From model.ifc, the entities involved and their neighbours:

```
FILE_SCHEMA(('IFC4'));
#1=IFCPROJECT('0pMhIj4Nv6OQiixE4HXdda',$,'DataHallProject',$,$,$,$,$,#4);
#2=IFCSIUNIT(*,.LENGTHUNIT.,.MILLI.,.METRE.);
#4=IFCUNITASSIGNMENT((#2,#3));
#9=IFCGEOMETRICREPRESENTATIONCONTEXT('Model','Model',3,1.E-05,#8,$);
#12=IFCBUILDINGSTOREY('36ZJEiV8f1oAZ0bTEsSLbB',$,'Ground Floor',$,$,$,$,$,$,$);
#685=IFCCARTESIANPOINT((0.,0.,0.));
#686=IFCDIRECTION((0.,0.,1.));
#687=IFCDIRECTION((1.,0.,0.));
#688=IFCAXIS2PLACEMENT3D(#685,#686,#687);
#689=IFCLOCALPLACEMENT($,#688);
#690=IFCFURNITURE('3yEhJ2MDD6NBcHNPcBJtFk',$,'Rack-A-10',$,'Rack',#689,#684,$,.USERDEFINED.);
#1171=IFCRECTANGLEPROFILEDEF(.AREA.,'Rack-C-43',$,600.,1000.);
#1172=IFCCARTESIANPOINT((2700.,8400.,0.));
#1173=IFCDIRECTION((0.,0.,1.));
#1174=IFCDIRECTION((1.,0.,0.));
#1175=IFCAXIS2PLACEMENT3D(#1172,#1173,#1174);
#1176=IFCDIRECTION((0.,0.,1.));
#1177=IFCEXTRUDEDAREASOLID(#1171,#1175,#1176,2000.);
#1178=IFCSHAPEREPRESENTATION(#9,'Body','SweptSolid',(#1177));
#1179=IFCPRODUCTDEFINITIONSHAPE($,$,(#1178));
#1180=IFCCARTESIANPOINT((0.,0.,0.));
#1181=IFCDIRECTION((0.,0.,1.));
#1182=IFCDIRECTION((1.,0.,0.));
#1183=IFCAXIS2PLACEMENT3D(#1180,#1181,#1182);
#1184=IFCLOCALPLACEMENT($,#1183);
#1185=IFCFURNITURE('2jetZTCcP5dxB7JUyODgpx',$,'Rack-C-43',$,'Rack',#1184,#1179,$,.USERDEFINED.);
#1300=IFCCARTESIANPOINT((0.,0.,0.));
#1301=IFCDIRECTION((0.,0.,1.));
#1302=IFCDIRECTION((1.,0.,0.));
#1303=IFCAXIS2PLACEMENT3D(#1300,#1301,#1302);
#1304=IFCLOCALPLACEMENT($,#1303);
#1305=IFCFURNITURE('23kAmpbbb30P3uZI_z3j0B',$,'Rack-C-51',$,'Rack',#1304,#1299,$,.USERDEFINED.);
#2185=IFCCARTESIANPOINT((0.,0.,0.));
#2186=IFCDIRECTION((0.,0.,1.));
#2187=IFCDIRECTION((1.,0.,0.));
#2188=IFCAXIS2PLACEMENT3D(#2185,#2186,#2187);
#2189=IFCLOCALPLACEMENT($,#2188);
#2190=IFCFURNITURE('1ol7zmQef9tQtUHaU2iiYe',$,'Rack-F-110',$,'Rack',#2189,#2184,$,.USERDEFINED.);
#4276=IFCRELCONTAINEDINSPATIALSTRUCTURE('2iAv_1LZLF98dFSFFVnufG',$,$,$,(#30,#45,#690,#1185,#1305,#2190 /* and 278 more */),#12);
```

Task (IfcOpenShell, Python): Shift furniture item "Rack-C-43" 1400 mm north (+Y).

```python
import ifcopenshell
import ifcopenshell.api.geometry
import ifcopenshell.util.placement
import ifcopenshell.util.unit

model = ifcopenshell.open("model.ifc")
unit_scale = ifcopenshell.util.unit.calculate_unit_scale(model)

item = model.by_guid("2jetZTCcP5dxB7JUyODgpx")
matrix = ifcopenshell.util.placement.get_local_placement(item.ObjectPlacement)
matrix[1, 3] += 1.4 / unit_scale
ifcopenshell.api.geometry.edit_object_placement(model, product=item, matrix=matrix, is_si=False)

print(ifcopenshell.util.placement.get_local_placement(item.ObjectPlacement).round(3) + 0.0)

model.write("model_edited.ifc")
```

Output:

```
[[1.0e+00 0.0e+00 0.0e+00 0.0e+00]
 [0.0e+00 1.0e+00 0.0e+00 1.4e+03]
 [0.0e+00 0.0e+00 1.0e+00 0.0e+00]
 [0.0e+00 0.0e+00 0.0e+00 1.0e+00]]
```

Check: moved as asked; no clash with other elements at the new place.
